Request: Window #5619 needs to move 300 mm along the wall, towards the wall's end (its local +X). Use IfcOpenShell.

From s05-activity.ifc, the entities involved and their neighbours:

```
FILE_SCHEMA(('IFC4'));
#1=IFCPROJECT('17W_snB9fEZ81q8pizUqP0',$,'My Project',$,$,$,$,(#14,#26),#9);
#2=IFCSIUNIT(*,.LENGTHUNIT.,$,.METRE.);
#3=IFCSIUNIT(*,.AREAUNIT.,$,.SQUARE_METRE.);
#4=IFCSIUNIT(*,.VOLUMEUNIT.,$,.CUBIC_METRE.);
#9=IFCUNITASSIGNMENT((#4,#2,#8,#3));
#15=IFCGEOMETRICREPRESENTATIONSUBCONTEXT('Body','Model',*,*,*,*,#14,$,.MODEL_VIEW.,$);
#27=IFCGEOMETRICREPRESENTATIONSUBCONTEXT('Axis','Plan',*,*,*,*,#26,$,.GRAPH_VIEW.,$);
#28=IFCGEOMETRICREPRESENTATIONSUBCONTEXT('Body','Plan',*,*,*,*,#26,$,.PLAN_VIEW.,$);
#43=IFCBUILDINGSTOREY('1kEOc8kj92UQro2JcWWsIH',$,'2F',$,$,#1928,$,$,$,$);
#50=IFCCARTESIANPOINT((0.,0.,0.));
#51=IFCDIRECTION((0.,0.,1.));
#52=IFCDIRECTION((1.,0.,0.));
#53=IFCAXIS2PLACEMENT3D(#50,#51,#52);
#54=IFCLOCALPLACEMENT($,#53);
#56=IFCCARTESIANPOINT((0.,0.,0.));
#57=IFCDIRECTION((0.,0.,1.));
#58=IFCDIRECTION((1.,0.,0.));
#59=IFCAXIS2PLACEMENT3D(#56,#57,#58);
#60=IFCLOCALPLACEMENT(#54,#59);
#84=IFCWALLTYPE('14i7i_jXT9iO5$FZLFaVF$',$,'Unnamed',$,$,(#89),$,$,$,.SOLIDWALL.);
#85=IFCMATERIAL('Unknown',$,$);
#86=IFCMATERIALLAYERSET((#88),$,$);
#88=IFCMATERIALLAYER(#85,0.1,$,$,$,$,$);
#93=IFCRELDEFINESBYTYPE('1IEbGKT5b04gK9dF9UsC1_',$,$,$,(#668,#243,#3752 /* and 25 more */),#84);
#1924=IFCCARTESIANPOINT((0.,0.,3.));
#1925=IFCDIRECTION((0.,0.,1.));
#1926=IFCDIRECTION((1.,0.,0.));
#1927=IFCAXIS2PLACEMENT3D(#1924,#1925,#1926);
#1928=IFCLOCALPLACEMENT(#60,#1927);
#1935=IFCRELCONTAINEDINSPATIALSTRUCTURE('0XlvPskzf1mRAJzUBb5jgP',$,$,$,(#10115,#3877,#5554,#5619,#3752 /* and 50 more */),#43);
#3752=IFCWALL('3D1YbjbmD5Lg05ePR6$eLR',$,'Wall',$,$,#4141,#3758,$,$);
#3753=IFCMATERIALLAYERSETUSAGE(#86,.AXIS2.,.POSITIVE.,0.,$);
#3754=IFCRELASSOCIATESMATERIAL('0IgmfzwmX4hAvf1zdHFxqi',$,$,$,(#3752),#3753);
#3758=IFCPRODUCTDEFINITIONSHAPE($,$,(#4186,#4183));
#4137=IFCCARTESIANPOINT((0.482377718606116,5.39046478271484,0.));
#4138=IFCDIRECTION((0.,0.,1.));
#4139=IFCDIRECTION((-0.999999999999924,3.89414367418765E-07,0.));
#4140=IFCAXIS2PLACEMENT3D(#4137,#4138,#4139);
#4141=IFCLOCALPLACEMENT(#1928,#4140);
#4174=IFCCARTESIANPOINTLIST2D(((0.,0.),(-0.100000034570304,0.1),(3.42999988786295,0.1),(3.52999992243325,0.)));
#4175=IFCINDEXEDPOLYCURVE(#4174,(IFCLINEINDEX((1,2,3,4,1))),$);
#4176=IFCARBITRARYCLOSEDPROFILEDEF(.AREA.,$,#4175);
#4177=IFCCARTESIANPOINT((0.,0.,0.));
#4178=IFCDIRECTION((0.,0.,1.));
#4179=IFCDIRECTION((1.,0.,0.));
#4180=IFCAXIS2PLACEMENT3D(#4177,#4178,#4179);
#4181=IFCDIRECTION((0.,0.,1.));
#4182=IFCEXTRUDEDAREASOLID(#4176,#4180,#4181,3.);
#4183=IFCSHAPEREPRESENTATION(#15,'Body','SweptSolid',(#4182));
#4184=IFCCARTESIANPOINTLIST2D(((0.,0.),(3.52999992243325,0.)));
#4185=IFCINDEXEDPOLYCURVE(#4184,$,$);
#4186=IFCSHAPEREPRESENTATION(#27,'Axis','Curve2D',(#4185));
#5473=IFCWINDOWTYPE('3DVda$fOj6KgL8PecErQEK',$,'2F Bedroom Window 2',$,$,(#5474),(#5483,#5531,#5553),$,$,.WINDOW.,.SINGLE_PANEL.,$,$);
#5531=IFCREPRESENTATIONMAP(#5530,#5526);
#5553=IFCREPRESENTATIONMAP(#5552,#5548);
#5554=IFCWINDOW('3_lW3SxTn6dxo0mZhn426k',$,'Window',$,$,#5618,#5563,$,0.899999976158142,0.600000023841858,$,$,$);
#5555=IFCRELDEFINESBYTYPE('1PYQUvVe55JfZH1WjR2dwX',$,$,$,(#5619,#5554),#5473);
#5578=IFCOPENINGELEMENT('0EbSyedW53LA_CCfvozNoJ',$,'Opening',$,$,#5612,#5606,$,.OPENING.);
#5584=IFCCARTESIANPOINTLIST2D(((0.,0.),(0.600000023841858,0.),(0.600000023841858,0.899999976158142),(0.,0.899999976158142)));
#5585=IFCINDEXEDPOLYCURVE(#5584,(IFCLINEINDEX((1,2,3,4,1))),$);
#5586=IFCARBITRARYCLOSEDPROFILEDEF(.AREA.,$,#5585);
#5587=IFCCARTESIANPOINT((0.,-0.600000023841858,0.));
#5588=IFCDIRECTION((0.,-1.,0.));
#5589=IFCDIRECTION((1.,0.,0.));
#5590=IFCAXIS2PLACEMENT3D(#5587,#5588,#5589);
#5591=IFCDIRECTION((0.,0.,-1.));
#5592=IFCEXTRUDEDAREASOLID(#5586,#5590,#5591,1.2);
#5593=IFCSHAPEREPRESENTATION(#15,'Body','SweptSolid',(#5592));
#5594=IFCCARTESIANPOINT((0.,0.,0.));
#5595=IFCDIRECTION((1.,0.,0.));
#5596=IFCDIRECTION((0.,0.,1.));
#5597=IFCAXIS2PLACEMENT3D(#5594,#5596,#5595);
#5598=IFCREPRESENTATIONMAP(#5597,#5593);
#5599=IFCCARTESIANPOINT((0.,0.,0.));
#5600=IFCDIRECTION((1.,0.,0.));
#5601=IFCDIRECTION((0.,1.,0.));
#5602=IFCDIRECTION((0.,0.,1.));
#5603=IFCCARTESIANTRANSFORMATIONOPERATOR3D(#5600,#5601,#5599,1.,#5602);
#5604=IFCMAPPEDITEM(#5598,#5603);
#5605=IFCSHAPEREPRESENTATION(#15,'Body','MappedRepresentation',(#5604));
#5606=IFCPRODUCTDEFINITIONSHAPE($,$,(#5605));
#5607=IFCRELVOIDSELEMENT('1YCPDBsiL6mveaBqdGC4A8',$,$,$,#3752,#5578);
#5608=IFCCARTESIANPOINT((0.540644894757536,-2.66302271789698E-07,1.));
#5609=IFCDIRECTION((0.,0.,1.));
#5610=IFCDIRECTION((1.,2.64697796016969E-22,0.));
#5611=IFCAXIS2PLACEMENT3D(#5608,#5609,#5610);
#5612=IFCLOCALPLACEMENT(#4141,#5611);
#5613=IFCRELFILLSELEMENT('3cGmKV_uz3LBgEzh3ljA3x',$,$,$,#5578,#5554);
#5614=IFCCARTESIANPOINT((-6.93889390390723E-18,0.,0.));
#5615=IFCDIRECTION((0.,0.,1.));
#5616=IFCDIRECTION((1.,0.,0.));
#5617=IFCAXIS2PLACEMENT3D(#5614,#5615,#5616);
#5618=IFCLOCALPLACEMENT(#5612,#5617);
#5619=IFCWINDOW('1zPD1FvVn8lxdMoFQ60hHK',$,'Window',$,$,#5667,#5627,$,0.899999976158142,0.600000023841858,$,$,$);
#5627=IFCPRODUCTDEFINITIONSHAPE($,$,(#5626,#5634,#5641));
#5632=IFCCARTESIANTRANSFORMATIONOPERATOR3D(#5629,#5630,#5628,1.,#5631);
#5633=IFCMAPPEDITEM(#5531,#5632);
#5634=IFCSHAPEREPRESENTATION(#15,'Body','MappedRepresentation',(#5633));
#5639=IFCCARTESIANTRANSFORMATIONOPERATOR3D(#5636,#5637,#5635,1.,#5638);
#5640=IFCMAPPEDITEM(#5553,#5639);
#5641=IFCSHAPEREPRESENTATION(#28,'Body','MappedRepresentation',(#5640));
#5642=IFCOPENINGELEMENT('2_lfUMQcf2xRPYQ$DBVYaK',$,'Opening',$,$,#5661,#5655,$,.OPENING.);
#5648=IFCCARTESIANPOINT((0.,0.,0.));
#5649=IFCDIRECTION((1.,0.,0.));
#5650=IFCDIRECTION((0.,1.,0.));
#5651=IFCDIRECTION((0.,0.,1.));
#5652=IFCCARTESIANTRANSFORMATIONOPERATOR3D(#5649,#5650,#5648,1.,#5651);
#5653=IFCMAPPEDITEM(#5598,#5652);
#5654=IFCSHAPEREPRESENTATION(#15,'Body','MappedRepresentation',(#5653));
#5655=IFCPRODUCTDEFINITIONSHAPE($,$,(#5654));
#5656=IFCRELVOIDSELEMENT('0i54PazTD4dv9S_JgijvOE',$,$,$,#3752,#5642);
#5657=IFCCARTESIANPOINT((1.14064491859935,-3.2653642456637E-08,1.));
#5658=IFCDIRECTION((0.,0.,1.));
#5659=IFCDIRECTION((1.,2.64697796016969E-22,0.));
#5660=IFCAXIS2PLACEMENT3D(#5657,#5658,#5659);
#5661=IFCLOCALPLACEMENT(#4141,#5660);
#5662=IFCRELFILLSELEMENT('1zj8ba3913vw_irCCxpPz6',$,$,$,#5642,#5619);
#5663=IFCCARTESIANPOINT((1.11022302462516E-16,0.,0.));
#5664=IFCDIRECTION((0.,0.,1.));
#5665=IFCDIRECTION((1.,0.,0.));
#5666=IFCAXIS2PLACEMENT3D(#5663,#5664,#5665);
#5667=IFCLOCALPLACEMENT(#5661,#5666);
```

```python
import ifcopenshell
import ifcopenshell.api.geometry
import ifcopenshell.util.placement

model = ifcopenshell.open("s05-activity.ifc")

window = model.by_id(5619)
opening = window.FillsVoids[0].RelatingOpeningElement
wall = opening.VoidsElements[0].RelatingBuildingElement

wall_matrix = ifcopenshell.util.placement.get_local_placement(wall.ObjectPlacement)
shift = wall_matrix[:3, 0] * 0.3
before = ifcopenshell.util.placement.get_local_placement(window.ObjectPlacement)[:3, 3].copy()

# The window is placed relative to its opening, so it follows when the opening moves.
matrix = ifcopenshell.util.placement.get_local_placement(opening.ObjectPlacement)
matrix[:3, 3] += shift
ifcopenshell.api.geometry.edit_object_placement(
    model, product=opening, matrix=matrix, is_si=False, should_transform_children=True
)

after = ifcopenshell.util.placement.get_local_placement(window.ObjectPlacement)[:3, 3]
print("window moved by", (after - before).round(3) + 0.0)

model.write("s05-activity_updated.ifc")
```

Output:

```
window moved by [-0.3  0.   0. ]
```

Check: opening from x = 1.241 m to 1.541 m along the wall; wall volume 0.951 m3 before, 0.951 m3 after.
